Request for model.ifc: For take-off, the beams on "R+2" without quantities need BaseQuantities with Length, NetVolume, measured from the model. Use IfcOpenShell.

First a look at what the model holds.

```python
import ifcopenshell
import ifcopenshell.util.element
import ifcopenshell.util.unit

model = ifcopenshell.open("model.ifc")
print(model.schema)
for unit_type in ("LENGTHUNIT", "AREAUNIT", "VOLUMEUNIT"):
    print(unit_type, ifcopenshell.util.unit.calculate_unit_scale(model, unit_type))
storey = next(s for s in model.by_type("IfcBuildingStorey") if s.Name == "R+2")
beams = [e for e in ifcopenshell.util.element.get_decomposition(storey) if e.is_a("IfcBeam")]
for e in sorted(beams, key=lambda e: e.id()):
    print(e.id(), e.is_a(), e.Name, list(ifcopenshell.util.element.get_psets(e, qtos_only=True)), sep=" | ")
```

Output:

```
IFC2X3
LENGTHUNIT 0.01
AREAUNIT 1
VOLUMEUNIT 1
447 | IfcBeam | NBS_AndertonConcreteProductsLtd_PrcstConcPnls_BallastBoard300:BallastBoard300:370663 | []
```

```python
import ifcopenshell
import ifcopenshell.api.pset
import ifcopenshell.geom
import ifcopenshell.util.element
import ifcopenshell.util.shape
import ifcopenshell.util.unit

model = ifcopenshell.open("model.ifc")
unit_scale = ifcopenshell.util.unit.calculate_unit_scale(model)
volume_scale = ifcopenshell.util.unit.calculate_unit_scale(model, "VOLUMEUNIT")
settings = ifcopenshell.geom.settings()

storey = next(s for s in model.by_type("IfcBuildingStorey") if s.Name == "R+2")
beams = [e for e in ifcopenshell.util.element.get_decomposition(storey) if e.is_a("IfcBeam")]

for e in sorted(beams, key=lambda e: e.id()):
    if ifcopenshell.util.element.get_psets(e, qtos_only=True, should_inherit=False):
        continue
    # Geometry comes back in metres, in the element's own axes.
    shape = ifcopenshell.geom.create_shape(settings, e)
    values = {
        "Length": ifcopenshell.util.shape.get_max_xyz(shape.geometry) / unit_scale,
        "NetVolume": ifcopenshell.util.shape.get_volume(shape.geometry) / volume_scale,
    }
    qto = ifcopenshell.api.pset.add_qto(model, product=e, name="BaseQuantities")
    ifcopenshell.api.pset.edit_qto(model, qto=qto, properties=values)
    print(e.id(), {k: round(v, 3) for k, v in values.items()})

model.write("model_v2.ifc")
```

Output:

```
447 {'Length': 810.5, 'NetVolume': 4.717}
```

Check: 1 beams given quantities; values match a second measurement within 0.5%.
